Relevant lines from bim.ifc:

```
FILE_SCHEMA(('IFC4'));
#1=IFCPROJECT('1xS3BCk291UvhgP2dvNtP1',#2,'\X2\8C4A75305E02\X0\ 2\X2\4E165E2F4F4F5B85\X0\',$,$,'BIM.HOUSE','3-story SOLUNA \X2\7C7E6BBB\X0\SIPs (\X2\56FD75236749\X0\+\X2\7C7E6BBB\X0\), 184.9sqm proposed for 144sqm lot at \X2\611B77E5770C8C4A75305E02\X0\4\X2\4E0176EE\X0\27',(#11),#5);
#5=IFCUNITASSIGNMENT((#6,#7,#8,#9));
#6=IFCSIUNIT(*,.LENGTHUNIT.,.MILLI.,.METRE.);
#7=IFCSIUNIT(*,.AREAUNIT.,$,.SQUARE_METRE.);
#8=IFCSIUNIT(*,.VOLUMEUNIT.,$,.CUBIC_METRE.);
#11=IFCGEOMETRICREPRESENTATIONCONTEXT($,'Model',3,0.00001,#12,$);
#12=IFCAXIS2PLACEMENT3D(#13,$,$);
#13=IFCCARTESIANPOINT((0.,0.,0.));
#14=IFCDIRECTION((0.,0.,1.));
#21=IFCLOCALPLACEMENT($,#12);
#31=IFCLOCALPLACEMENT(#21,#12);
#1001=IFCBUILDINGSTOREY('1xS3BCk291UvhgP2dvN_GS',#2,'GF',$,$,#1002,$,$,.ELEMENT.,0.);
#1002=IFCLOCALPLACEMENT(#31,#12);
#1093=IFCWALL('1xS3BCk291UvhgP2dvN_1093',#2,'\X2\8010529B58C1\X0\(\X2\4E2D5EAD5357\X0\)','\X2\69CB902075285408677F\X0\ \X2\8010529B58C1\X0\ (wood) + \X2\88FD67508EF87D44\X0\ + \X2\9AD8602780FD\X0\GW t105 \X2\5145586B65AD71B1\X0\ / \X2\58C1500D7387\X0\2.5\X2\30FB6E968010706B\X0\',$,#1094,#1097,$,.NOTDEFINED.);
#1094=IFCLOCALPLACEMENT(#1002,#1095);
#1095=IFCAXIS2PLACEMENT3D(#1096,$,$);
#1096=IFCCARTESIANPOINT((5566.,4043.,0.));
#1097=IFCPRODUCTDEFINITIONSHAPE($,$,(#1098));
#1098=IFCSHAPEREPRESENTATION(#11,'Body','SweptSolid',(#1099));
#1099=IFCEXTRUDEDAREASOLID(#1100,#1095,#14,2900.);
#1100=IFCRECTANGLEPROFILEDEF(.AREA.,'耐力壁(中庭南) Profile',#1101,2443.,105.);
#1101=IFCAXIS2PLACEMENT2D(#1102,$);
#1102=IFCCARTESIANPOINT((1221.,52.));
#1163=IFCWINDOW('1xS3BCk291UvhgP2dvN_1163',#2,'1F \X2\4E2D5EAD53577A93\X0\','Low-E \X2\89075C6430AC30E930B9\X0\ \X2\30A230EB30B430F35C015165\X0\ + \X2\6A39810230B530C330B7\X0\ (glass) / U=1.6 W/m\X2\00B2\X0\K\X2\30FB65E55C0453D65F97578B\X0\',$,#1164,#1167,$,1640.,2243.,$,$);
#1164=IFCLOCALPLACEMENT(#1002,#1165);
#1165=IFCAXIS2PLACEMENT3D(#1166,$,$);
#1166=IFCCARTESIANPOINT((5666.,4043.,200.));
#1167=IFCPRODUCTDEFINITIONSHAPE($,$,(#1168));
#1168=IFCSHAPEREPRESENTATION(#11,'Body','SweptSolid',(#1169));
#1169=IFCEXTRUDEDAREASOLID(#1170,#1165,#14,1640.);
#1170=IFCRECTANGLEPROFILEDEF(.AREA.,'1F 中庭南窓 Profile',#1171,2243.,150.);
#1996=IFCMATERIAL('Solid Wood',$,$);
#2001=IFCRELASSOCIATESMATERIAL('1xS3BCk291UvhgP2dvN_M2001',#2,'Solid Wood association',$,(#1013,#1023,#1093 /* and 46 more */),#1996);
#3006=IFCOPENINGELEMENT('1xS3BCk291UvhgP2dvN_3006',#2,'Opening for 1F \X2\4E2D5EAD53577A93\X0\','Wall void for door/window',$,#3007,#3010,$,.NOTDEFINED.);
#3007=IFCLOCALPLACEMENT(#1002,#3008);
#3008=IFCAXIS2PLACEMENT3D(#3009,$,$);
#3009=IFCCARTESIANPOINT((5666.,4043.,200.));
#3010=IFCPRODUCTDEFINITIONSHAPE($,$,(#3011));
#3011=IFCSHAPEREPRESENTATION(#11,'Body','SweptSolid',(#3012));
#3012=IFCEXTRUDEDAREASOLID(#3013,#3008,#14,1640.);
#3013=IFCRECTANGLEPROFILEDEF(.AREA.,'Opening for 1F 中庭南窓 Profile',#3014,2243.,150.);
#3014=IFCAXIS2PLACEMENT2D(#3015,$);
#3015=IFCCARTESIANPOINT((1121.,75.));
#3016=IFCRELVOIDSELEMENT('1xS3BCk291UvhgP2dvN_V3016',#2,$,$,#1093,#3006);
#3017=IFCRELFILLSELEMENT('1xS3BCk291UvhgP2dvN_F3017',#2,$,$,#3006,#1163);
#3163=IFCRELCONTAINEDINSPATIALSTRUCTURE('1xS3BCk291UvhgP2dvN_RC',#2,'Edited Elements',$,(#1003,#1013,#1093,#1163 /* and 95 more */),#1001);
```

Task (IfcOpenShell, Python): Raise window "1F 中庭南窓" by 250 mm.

```python
import numpy as np
import ifcopenshell
import ifcopenshell.api.geometry
import ifcopenshell.util.placement
import ifcopenshell.util.unit

model = ifcopenshell.open("bim.ifc")
unit_scale = ifcopenshell.util.unit.calculate_unit_scale(model)

window = model.by_guid("1xS3BCk291UvhgP2dvN_1163")
opening = window.FillsVoids[0].RelatingOpeningElement
dz = 0.25 / unit_scale

shift = np.array([0.0, 0.0, dz])
# The window is not placed relative to its opening, so move both.
for product in (opening, window):
    matrix = ifcopenshell.util.placement.get_local_placement(product.ObjectPlacement)
    matrix[:3, 3] += shift
    ifcopenshell.api.geometry.edit_object_placement(model, product=product, matrix=matrix, is_si=False)

print(f"moved by {dz * unit_scale:+.3f} m")

model.write("bim-out.ifc")
```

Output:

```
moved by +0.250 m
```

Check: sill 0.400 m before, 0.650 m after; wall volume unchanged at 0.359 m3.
